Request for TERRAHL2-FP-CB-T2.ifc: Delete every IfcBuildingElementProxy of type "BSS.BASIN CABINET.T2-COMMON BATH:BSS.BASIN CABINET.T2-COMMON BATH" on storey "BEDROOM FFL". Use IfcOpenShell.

First a look at what the model holds.

```python
import ifcopenshell
import ifcopenshell.util.element

model = ifcopenshell.open("TERRAHL2-FP-CB-T2.ifc")
print(model.schema)
storey = next(s for s in model.by_type("IfcBuildingStorey") if s.Name == "BEDROOM FFL")
proxies = [e for e in ifcopenshell.util.element.get_decomposition(storey) if e.is_a("IfcBuildingElementProxy")]
seen = {}
for e in proxies:
    element_type = ifcopenshell.util.element.get_type(e)
    name = element_type.Name if element_type not in (None, e) else None
    seen[name] = seen.get(name, 0) + 1
for name, count in sorted(seen.items(), key=str):
    print(count, "x", name)
```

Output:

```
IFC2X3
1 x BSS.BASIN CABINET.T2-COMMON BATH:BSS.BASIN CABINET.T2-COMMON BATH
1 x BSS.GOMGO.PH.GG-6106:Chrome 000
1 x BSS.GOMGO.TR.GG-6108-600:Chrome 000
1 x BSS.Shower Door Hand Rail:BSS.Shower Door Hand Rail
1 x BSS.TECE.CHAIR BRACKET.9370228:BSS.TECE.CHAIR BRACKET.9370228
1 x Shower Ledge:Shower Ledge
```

```python
import ifcopenshell
import ifcopenshell.api.root
import ifcopenshell.util.element

model = ifcopenshell.open("TERRAHL2-FP-CB-T2.ifc")

storey = next(s for s in model.by_type("IfcBuildingStorey") if s.Name == "BEDROOM FFL")
proxies = [e for e in ifcopenshell.util.element.get_decomposition(storey) if e.is_a("IfcBuildingElementProxy")]
targets = [e for e in proxies if (t := ifcopenshell.util.element.get_type(e)) not in (None, e) and t.Name == "BSS.BASIN CABINET.T2-COMMON BATH:BSS.BASIN CABINET.T2-COMMON BATH"]

for e in targets:
    ifcopenshell.api.root.remove_product(model, product=e)
print(len(targets), "removed")

model.write("TERRAHL2-FP-CB-T2_rev.ifc")
```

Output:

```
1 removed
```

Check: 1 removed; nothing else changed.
